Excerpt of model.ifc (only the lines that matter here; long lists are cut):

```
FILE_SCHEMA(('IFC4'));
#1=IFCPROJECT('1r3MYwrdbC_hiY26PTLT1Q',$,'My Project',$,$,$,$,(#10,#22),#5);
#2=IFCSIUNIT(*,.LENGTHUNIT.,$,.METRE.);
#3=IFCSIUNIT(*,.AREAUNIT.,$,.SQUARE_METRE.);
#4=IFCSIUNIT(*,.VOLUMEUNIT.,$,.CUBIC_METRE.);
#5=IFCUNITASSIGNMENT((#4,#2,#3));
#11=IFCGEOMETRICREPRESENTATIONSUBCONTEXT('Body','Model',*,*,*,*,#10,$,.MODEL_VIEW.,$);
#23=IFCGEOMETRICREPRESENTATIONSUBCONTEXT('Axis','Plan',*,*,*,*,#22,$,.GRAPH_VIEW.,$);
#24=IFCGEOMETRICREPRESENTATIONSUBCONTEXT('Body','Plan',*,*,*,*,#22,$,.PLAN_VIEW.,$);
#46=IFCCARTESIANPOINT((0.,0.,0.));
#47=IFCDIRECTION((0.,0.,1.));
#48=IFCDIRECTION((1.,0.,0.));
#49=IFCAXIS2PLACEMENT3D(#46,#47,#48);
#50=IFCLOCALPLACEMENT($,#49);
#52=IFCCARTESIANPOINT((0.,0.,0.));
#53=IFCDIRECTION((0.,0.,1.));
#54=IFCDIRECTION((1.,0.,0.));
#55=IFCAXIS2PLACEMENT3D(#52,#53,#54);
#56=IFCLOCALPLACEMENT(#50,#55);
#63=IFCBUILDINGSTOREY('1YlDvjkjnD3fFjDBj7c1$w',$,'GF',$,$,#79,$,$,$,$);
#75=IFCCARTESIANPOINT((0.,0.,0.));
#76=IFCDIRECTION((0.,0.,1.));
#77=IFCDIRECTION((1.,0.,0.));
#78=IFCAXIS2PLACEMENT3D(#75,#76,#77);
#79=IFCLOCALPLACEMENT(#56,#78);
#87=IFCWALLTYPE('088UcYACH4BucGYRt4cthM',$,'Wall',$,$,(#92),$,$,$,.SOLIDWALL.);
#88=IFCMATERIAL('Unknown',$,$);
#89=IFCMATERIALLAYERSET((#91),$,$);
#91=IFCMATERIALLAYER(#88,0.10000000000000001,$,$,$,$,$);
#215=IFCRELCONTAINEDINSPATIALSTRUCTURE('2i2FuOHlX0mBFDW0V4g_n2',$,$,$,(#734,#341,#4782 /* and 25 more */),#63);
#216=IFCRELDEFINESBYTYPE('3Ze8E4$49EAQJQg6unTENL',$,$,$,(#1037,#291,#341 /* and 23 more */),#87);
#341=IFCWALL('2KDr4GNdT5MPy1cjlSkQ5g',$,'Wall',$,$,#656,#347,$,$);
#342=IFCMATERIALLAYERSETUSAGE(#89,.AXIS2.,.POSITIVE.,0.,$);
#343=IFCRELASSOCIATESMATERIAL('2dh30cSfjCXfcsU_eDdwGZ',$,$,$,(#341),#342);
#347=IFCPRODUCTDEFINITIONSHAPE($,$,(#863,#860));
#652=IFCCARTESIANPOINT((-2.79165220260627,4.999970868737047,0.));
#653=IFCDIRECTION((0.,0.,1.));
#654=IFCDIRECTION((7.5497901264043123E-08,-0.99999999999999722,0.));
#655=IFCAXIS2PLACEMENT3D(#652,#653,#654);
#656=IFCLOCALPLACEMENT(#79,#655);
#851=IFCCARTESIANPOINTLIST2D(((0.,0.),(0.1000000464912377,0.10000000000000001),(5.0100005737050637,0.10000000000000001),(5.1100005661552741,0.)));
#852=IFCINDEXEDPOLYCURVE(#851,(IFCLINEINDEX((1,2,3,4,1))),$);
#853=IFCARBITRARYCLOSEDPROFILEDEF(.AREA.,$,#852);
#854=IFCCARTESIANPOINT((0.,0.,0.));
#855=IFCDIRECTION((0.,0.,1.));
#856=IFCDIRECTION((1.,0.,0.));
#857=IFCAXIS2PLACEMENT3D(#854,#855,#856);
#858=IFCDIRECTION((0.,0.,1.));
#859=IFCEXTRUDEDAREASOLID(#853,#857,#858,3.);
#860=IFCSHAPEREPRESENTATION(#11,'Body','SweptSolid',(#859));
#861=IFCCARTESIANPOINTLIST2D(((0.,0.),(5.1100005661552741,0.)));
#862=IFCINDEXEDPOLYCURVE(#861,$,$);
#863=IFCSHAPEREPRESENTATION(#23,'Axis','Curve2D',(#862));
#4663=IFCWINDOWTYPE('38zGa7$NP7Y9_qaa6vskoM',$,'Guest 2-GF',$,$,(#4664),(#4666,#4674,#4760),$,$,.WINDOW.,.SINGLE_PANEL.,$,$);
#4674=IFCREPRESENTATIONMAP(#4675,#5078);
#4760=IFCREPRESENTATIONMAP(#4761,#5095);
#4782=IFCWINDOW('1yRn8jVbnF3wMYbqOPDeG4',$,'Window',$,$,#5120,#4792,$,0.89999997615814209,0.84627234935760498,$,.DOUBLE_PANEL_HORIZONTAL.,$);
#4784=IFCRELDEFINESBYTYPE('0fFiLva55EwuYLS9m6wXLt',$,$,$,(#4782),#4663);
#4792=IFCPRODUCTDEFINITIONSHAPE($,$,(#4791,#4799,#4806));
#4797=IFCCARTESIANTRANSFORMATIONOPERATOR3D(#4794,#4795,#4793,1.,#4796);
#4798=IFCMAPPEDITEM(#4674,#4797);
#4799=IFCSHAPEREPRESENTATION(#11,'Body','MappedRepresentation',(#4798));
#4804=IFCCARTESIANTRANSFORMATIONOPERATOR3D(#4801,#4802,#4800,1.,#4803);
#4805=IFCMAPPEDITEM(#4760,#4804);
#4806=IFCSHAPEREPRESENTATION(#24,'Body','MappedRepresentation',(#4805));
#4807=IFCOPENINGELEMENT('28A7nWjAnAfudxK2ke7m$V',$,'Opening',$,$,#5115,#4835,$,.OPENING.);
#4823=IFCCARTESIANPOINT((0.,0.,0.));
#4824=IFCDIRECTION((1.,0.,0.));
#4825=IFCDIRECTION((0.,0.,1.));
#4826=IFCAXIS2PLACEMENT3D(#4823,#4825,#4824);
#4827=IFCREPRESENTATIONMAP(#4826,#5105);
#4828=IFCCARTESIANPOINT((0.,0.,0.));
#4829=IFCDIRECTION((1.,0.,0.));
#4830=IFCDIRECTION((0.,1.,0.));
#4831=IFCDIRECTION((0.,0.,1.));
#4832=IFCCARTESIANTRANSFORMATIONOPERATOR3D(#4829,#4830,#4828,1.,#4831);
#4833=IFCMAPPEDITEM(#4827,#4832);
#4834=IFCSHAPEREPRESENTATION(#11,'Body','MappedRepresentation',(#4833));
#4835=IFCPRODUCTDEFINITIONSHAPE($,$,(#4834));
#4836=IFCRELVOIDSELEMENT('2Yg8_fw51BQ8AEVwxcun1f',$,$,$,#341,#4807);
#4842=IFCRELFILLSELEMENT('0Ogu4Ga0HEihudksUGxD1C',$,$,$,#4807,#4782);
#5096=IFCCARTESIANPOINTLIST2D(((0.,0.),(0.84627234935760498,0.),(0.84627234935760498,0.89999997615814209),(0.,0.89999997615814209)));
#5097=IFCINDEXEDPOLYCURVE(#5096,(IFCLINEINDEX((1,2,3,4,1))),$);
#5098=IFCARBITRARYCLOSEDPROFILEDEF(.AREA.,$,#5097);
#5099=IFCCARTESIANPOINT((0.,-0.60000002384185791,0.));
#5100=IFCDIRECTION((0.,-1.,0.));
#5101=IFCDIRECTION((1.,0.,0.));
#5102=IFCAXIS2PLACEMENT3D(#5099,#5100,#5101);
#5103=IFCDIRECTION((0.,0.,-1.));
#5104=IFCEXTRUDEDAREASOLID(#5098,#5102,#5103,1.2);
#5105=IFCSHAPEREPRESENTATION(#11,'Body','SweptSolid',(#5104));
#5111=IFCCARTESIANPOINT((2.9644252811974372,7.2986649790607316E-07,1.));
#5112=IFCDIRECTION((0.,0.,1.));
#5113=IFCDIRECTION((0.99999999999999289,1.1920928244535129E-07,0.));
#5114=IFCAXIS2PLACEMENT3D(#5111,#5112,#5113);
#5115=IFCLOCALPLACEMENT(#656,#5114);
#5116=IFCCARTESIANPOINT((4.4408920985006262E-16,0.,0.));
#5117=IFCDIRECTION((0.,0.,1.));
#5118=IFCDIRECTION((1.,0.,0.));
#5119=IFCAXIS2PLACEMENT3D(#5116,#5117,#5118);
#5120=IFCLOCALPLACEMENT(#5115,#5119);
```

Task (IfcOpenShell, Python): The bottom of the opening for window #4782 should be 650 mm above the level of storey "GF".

```python
import numpy as np
import ifcopenshell
import ifcopenshell.api.geometry
import ifcopenshell.geom
import ifcopenshell.util.element
import ifcopenshell.util.placement
import ifcopenshell.util.shape
import ifcopenshell.util.unit

model = ifcopenshell.open("model.ifc")
unit_scale = ifcopenshell.util.unit.calculate_unit_scale(model)

window = model.by_guid("1yRn8jVbnF3wMYbqOPDeG4")
opening = window.FillsVoids[0].RelatingOpeningElement
storey = ifcopenshell.util.element.get_container(window, ifc_class="IfcBuildingStorey")
level = ifcopenshell.util.placement.get_local_placement(storey.ObjectPlacement)[2, 3]

# The opening's origin need not be at the sill, so measure its lowest point.
shape = ifcopenshell.geom.create_shape(ifcopenshell.geom.settings(), opening)
bottom = ifcopenshell.util.shape.get_shape_bottom_elevation(shape, shape.geometry) / unit_scale
dz = level + 0.65 / unit_scale - bottom

shift = np.array([0.0, 0.0, dz])
# The window is placed relative to its opening, so it follows when the opening moves.
matrix = ifcopenshell.util.placement.get_local_placement(opening.ObjectPlacement)
matrix[:3, 3] += shift
ifcopenshell.api.geometry.edit_object_placement(
    model, product=opening, matrix=matrix, is_si=False, should_transform_children=True
)

print(f"moved by {dz * unit_scale:+.3f} m")

model.write("model_updated.ifc")
```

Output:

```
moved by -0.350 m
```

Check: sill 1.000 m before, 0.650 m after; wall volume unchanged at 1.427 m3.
